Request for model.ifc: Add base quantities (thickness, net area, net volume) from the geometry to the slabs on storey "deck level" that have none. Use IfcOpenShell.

First a look at what the model holds.

```python
import ifcopenshell
import ifcopenshell.util.element
import ifcopenshell.util.unit

model = ifcopenshell.open("model.ifc")
print(model.schema)
for unit_type in ("LENGTHUNIT", "AREAUNIT", "VOLUMEUNIT"):
    print(unit_type, ifcopenshell.util.unit.calculate_unit_scale(model, unit_type))
storey = next(s for s in model.by_type("IfcBuildingStorey") if s.Name == "deck level")
slabs = [e for e in ifcopenshell.util.element.get_decomposition(storey) if e.is_a("IfcSlab")]
for e in sorted(slabs, key=lambda e: e.id()):
    print(e.id(), e.is_a(), e.Name, list(ifcopenshell.util.element.get_psets(e, qtos_only=True)), sep=" | ")
```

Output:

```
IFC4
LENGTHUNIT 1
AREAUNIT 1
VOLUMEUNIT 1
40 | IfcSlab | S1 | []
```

```python
import ifcopenshell
import ifcopenshell.api.pset
import ifcopenshell.geom
import ifcopenshell.util.element
import ifcopenshell.util.shape
import ifcopenshell.util.unit

model = ifcopenshell.open("model.ifc")
unit_scale = ifcopenshell.util.unit.calculate_unit_scale(model)
area_scale = ifcopenshell.util.unit.calculate_unit_scale(model, "AREAUNIT")
volume_scale = ifcopenshell.util.unit.calculate_unit_scale(model, "VOLUMEUNIT")
settings = ifcopenshell.geom.settings()

storey = next(s for s in model.by_type("IfcBuildingStorey") if s.Name == "deck level")
slabs = [e for e in ifcopenshell.util.element.get_decomposition(storey) if e.is_a("IfcSlab")]

for e in sorted(slabs, key=lambda e: e.id()):
    if ifcopenshell.util.element.get_psets(e, qtos_only=True, should_inherit=False):
        continue
    # Geometry comes back in metres, in the element's own axes.
    shape = ifcopenshell.geom.create_shape(settings, e)
    values = {
        "Width": ifcopenshell.util.shape.get_z(shape.geometry) / unit_scale,
        "NetArea": ifcopenshell.util.shape.get_footprint_area(shape.geometry) / area_scale,
        "NetVolume": ifcopenshell.util.shape.get_volume(shape.geometry) / volume_scale,
    }
    qto = ifcopenshell.api.pset.add_qto(model, product=e, name="Qto_SlabBaseQuantities")
    ifcopenshell.api.pset.edit_qto(model, qto=qto, properties=values)
    print(e.id(), {k: round(v, 3) for k, v in values.items()})

model.write("model_rev.ifc")
```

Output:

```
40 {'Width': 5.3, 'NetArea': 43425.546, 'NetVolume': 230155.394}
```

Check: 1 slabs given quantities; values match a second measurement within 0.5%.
